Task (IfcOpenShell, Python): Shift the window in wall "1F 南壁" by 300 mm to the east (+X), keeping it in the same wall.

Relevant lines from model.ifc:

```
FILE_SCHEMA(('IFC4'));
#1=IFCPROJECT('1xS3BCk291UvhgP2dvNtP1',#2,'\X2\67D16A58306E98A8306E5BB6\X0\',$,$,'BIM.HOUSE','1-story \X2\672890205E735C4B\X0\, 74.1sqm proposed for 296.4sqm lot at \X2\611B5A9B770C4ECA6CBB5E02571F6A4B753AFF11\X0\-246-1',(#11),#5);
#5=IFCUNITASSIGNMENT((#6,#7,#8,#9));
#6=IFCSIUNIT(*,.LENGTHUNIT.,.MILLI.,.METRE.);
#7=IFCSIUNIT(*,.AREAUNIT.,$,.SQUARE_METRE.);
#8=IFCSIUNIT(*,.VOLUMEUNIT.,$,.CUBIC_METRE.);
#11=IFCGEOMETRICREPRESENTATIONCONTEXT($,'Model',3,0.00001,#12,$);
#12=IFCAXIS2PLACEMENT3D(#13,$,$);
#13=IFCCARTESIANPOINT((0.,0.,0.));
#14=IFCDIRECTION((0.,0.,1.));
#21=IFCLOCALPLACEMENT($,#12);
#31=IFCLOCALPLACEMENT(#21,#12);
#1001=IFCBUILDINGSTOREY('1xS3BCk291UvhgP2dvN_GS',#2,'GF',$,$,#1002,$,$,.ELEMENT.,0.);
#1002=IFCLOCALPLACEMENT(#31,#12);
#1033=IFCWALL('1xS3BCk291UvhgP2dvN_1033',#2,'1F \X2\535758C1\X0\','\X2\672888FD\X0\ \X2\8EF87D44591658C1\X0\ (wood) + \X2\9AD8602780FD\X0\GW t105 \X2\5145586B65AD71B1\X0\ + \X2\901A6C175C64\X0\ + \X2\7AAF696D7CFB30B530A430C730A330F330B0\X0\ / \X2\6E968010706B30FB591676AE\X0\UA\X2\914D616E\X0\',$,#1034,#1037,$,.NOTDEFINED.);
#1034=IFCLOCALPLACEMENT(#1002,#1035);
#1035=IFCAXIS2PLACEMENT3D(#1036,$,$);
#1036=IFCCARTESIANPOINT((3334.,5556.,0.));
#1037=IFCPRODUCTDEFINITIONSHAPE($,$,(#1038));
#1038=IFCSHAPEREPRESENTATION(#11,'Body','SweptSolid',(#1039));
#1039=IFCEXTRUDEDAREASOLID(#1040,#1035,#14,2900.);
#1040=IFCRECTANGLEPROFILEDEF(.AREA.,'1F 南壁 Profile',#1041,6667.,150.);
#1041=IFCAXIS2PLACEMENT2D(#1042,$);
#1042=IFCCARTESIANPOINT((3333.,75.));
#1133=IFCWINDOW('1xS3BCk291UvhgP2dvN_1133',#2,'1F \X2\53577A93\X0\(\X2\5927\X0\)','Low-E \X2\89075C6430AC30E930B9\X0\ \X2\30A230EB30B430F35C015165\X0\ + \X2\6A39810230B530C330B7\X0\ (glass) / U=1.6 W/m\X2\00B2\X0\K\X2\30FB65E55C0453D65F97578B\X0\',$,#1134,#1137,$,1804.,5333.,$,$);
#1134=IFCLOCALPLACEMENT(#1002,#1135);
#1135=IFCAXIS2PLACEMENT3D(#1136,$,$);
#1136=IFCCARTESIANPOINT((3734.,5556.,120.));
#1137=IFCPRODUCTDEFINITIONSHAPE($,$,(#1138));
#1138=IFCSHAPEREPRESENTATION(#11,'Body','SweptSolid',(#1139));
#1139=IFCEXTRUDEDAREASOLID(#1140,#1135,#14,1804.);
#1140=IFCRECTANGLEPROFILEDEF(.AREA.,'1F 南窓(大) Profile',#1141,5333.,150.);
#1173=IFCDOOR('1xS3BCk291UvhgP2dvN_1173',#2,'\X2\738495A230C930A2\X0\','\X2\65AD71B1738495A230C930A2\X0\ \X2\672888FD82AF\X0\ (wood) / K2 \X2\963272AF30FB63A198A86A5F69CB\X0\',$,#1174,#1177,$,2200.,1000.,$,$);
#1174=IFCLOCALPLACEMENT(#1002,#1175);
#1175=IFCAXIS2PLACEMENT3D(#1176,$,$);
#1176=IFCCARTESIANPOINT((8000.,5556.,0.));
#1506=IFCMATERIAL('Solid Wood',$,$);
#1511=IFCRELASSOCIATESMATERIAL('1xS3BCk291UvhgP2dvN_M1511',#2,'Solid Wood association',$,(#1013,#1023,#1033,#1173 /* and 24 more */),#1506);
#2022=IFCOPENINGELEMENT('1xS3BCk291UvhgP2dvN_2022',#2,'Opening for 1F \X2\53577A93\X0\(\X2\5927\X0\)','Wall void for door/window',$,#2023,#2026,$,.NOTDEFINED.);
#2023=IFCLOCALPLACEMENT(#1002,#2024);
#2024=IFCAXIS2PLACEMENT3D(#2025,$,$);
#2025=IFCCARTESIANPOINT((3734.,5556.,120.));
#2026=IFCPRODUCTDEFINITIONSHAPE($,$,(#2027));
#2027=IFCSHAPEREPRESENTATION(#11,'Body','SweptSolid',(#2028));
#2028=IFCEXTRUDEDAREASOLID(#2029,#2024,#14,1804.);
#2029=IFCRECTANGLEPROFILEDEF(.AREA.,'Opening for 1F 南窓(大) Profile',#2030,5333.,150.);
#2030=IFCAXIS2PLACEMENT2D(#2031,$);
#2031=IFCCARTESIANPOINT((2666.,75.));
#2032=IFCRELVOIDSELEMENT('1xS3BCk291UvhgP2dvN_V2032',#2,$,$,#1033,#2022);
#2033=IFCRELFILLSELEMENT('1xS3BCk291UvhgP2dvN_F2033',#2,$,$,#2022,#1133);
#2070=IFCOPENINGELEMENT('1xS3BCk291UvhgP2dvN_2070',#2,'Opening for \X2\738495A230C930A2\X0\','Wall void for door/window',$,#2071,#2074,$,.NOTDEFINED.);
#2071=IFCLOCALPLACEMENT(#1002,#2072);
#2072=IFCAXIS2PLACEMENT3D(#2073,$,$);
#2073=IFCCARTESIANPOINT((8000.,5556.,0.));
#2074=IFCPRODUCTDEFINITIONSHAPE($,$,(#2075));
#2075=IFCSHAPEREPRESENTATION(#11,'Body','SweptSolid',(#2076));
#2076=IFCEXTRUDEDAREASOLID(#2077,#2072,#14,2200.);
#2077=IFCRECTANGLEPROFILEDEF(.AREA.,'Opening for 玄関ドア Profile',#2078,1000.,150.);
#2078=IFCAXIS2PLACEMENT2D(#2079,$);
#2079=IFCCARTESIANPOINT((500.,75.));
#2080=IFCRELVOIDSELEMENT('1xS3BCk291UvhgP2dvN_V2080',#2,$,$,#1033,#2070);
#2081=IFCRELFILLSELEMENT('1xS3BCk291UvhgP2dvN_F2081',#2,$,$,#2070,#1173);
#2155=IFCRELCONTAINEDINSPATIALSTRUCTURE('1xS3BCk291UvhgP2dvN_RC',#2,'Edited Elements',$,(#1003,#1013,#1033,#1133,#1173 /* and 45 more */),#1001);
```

```python
import ifcopenshell
import ifcopenshell.api.geometry
import ifcopenshell.util.placement
import ifcopenshell.util.unit

model = ifcopenshell.open("model.ifc")
unit_scale = ifcopenshell.util.unit.calculate_unit_scale(model)

window = model.by_guid("1xS3BCk291UvhgP2dvN_1133")
opening = window.FillsVoids[0].RelatingOpeningElement
wall = opening.VoidsElements[0].RelatingBuildingElement

wall_matrix = ifcopenshell.util.placement.get_local_placement(wall.ObjectPlacement)
shift = wall_matrix[:3, 0] * 0.3 / unit_scale
before = ifcopenshell.util.placement.get_local_placement(window.ObjectPlacement)[:3, 3].copy()

# The window is not placed relative to its opening, so move both.
for product in (opening, window):
    matrix = ifcopenshell.util.placement.get_local_placement(product.ObjectPlacement)
    matrix[:3, 3] += shift
    ifcopenshell.api.geometry.edit_object_placement(model, product=product, matrix=matrix, is_si=False)

after = ifcopenshell.util.placement.get_local_placement(window.ObjectPlacement)[:3, 3]
print("window moved by", (after - before).round(3) + 0.0)

model.write("model_updated.ifc")
```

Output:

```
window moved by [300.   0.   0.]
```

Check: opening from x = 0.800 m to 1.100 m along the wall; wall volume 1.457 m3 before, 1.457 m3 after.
